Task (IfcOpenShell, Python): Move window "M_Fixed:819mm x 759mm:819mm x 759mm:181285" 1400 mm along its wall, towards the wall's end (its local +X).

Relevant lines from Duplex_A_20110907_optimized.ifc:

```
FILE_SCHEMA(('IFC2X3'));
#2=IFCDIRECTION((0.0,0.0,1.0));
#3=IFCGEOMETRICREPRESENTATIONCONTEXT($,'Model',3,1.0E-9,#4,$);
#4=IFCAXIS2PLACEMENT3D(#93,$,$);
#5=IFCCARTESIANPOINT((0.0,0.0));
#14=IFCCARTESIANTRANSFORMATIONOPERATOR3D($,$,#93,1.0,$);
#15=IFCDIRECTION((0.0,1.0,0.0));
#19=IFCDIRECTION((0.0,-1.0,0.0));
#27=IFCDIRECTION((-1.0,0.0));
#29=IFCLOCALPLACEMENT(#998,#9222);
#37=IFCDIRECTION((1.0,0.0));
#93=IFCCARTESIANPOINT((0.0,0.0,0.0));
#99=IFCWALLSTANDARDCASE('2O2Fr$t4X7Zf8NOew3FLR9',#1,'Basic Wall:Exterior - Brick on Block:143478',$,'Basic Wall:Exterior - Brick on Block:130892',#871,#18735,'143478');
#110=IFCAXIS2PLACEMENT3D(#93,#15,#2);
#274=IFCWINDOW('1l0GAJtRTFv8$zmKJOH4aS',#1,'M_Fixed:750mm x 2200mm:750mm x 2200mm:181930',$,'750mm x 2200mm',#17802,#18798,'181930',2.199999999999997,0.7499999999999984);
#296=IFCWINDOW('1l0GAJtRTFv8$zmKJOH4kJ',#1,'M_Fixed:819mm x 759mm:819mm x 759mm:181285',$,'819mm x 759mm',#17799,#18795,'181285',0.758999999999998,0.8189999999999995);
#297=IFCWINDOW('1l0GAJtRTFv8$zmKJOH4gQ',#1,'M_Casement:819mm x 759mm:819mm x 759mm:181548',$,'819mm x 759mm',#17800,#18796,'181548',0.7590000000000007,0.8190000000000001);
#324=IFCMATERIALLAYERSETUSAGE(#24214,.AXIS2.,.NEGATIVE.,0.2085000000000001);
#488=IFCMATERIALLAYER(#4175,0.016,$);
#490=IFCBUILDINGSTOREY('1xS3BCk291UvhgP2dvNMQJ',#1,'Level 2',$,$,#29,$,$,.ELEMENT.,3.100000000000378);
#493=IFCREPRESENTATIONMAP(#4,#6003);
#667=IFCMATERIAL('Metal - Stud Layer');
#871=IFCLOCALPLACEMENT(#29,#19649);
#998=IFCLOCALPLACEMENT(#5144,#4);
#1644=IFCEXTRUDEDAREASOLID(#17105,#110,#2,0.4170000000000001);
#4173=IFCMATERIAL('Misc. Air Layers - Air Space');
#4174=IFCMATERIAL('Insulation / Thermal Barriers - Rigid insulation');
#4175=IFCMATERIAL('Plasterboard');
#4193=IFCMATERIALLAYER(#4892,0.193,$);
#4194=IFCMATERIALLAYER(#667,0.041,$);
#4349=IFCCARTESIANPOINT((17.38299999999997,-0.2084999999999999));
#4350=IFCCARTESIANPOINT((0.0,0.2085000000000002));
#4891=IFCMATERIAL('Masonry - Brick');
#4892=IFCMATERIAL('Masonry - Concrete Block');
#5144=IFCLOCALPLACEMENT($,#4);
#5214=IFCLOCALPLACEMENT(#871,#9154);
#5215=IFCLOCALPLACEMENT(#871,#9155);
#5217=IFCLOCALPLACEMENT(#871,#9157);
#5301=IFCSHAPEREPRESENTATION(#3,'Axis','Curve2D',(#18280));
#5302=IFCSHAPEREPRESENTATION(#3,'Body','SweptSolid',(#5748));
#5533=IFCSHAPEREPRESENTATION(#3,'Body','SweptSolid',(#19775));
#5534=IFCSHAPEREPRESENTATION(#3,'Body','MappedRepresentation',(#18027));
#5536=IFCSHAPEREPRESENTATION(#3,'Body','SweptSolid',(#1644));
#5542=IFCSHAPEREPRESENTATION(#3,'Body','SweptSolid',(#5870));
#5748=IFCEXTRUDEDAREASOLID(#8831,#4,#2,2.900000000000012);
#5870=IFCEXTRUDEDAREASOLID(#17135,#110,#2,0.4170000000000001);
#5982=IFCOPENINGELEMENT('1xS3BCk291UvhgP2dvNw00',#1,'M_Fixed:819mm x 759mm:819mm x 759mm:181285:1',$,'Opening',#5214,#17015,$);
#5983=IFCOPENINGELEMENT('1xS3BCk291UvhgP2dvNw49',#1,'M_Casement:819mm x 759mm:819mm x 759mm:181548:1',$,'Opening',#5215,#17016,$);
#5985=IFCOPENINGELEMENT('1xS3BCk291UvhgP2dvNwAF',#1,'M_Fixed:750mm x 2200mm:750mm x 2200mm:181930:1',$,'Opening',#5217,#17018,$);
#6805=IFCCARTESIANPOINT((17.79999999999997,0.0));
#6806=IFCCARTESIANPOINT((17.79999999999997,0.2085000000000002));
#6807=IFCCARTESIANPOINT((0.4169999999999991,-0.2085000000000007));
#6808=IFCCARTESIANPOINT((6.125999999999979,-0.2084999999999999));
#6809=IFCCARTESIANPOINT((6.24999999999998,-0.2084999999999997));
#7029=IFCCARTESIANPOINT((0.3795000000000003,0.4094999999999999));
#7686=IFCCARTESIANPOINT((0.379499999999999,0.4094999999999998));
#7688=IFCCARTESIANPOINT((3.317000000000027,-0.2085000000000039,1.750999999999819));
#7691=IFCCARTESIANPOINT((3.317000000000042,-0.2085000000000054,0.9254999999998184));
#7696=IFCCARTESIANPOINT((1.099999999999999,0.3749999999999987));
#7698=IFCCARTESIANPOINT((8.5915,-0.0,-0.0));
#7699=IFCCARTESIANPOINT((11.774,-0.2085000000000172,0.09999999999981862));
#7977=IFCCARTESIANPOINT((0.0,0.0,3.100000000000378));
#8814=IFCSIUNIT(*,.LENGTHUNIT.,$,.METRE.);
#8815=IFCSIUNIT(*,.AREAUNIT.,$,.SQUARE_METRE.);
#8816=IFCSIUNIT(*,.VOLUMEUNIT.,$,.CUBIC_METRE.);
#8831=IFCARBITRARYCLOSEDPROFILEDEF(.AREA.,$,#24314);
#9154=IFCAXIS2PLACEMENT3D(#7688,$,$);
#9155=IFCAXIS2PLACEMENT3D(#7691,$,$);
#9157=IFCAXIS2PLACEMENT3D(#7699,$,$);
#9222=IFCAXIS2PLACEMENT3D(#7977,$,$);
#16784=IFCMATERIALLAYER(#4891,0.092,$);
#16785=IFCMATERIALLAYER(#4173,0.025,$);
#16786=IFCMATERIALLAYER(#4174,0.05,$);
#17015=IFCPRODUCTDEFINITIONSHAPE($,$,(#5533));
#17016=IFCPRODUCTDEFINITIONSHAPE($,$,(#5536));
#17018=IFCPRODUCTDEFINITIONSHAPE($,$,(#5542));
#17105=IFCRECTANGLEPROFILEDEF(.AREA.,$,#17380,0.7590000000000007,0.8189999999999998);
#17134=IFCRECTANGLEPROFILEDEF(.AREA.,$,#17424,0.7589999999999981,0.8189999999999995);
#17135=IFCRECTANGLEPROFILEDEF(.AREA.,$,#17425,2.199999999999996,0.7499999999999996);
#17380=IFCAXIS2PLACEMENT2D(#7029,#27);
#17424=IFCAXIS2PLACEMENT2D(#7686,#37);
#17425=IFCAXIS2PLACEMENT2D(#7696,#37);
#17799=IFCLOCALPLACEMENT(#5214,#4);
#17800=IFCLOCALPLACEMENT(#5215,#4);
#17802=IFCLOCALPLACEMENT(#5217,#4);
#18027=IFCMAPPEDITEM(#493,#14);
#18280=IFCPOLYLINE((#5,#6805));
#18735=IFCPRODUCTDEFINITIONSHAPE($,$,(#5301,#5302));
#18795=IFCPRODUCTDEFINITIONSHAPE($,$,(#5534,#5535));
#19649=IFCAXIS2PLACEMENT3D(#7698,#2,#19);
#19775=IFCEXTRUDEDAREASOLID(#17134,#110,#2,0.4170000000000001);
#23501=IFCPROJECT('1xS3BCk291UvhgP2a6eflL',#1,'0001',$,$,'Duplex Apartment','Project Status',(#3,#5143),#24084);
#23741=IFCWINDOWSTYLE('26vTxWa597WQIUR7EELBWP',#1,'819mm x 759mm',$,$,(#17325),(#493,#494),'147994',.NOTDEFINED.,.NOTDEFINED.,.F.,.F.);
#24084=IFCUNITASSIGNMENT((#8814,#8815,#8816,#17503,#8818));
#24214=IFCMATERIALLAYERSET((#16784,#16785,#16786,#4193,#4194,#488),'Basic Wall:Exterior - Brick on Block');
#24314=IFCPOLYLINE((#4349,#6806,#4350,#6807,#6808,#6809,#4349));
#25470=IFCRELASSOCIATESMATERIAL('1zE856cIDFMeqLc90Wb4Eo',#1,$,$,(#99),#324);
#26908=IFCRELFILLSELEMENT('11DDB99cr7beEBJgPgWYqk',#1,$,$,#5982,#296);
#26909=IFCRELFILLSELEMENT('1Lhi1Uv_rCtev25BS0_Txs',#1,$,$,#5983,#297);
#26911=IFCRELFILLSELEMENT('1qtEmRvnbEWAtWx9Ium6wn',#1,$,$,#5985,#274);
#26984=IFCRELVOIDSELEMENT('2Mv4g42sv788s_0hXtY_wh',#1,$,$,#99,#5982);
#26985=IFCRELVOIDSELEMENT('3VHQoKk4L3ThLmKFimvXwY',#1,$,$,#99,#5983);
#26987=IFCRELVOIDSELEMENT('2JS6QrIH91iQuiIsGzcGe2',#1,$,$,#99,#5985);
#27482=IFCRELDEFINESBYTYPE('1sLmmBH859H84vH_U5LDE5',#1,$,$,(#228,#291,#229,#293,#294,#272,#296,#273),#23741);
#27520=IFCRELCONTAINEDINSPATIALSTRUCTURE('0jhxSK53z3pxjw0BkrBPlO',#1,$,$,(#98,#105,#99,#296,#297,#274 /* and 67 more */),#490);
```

```python
import ifcopenshell
import ifcopenshell.api.geometry
import ifcopenshell.util.placement

model = ifcopenshell.open("Duplex_A_20110907_optimized.ifc")

window = model.by_guid("1l0GAJtRTFv8$zmKJOH4kJ")
opening = window.FillsVoids[0].RelatingOpeningElement
wall = opening.VoidsElements[0].RelatingBuildingElement

wall_matrix = ifcopenshell.util.placement.get_local_placement(wall.ObjectPlacement)
shift = wall_matrix[:3, 0] * 1.4
before = ifcopenshell.util.placement.get_local_placement(window.ObjectPlacement)[:3, 3].copy()

# The window is placed relative to its opening, so it follows when the opening moves.
matrix = ifcopenshell.util.placement.get_local_placement(opening.ObjectPlacement)
matrix[:3, 3] += shift
ifcopenshell.api.geometry.edit_object_placement(
    model, product=opening, matrix=matrix, is_si=False, should_transform_children=True
)

after = ifcopenshell.util.placement.get_local_placement(window.ObjectPlacement)[:3, 3]
print("window moved by", (after - before).round(3) + 0.0)

model.write("Duplex_A_20110907_optimized_rev.ifc")
```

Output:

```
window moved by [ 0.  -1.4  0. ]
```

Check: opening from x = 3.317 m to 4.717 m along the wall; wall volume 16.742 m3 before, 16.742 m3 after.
